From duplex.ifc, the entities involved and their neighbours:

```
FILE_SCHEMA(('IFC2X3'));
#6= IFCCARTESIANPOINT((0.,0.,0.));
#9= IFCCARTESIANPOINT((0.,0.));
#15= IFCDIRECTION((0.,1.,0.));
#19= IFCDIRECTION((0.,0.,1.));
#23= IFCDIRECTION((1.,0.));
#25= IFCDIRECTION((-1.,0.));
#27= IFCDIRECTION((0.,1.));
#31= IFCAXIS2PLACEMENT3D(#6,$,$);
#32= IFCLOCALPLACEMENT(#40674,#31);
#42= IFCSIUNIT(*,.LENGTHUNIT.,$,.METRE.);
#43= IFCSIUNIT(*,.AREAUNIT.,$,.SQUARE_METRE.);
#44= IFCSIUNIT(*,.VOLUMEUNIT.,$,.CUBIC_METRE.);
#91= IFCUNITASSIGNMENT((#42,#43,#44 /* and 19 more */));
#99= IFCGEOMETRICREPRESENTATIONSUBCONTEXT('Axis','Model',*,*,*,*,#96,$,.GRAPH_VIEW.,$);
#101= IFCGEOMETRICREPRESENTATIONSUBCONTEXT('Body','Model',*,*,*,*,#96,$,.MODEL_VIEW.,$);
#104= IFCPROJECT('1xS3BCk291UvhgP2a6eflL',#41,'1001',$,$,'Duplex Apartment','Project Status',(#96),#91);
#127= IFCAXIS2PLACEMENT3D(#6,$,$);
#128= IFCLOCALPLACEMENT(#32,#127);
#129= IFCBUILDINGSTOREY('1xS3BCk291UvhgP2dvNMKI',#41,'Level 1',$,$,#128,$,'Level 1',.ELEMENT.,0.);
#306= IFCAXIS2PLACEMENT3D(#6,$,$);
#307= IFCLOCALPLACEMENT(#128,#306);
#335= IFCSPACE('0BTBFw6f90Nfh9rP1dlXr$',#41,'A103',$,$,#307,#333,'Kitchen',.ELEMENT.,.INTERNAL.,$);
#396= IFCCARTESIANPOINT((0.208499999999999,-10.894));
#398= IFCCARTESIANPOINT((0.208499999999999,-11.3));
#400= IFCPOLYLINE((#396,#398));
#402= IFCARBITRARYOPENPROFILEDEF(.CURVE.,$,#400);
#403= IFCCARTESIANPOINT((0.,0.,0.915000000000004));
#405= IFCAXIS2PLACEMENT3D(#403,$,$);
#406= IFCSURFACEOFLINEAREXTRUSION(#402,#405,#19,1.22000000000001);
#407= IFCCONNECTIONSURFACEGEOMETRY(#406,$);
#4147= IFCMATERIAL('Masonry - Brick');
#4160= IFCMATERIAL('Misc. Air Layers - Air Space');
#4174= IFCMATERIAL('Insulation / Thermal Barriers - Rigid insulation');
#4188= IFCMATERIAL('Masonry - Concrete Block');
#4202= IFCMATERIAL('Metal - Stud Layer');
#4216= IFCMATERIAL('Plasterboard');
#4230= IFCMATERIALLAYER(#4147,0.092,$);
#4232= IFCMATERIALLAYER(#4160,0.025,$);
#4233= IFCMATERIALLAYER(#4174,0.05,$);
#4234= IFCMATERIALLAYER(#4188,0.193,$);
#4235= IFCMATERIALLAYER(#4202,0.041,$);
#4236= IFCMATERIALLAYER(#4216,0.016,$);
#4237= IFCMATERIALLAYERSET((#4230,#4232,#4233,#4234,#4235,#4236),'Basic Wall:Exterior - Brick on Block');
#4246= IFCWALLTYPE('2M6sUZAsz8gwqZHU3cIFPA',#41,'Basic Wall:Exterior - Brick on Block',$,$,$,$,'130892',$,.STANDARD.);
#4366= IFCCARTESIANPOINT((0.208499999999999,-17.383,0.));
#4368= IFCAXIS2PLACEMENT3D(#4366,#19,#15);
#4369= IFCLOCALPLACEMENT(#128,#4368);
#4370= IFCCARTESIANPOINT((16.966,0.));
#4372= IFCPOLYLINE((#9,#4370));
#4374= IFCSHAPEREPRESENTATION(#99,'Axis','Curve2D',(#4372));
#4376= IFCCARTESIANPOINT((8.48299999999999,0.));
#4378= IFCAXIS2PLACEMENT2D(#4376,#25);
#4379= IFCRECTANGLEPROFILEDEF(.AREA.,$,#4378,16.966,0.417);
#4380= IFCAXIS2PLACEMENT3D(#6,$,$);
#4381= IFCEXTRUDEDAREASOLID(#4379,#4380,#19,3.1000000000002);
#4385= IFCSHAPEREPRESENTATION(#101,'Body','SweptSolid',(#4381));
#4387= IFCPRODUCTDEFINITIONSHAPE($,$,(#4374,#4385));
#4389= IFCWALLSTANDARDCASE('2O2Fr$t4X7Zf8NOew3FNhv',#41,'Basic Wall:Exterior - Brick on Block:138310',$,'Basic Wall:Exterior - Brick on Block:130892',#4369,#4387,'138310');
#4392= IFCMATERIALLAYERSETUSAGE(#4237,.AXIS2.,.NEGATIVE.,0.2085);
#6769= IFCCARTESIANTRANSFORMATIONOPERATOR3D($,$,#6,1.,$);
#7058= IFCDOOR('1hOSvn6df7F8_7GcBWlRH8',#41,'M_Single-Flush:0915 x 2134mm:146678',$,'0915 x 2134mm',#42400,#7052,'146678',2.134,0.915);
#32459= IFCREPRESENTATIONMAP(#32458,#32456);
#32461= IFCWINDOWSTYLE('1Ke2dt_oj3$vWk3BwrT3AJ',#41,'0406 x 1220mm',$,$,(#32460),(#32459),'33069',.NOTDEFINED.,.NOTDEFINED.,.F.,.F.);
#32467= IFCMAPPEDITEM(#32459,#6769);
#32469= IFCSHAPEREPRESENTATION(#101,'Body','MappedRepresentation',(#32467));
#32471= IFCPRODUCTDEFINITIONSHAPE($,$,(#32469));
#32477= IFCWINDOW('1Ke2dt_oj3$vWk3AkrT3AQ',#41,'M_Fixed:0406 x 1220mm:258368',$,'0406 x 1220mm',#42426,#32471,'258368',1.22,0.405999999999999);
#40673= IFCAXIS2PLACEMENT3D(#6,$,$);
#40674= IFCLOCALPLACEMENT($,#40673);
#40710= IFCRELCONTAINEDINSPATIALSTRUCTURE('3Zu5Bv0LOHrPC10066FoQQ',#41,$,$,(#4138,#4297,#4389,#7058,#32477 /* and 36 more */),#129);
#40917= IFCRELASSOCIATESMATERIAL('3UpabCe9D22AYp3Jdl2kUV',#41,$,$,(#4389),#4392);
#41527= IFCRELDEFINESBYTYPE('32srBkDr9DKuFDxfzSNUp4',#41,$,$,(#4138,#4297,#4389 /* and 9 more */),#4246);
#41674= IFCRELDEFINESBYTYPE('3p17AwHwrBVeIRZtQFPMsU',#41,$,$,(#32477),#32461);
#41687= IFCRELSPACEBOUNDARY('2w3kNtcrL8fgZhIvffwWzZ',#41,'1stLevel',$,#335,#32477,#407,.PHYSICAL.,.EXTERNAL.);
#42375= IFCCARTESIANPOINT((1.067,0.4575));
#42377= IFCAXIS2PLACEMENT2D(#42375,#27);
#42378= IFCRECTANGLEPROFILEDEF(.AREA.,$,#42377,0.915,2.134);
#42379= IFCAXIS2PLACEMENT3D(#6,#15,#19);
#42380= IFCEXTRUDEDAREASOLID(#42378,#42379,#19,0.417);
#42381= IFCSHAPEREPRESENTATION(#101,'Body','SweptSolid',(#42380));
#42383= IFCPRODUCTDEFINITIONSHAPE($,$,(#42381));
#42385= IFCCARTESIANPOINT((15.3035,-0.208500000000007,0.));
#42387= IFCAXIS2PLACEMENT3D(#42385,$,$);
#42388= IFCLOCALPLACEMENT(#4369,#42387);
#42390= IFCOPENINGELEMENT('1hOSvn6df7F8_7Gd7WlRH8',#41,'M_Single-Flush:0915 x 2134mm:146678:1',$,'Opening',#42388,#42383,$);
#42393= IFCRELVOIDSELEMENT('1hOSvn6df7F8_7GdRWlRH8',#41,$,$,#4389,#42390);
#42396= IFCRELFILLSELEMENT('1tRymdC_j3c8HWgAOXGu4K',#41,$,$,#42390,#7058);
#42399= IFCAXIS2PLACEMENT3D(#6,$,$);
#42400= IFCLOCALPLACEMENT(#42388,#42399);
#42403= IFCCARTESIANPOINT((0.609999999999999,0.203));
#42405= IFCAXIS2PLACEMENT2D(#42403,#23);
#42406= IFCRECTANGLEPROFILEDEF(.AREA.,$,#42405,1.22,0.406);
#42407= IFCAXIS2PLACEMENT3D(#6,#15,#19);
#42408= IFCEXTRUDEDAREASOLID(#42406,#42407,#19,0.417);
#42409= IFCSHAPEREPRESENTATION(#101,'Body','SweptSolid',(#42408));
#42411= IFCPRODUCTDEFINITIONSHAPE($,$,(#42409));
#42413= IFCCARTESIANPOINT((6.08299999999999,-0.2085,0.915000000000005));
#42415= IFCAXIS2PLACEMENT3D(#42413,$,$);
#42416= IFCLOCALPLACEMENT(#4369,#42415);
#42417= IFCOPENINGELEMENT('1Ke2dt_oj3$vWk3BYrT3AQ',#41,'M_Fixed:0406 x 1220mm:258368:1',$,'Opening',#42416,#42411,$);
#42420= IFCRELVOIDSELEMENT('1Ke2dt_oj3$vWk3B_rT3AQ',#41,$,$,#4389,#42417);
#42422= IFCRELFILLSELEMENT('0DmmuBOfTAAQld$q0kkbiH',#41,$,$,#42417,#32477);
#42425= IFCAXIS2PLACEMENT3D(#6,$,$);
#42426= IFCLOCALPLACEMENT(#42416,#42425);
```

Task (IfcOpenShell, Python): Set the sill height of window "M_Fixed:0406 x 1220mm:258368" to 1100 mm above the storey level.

```python
import numpy as np
import ifcopenshell
import ifcopenshell.api.geometry
import ifcopenshell.geom
import ifcopenshell.util.element
import ifcopenshell.util.placement
import ifcopenshell.util.shape
import ifcopenshell.util.unit

model = ifcopenshell.open("duplex.ifc")
unit_scale = ifcopenshell.util.unit.calculate_unit_scale(model)

window = model.by_guid("1Ke2dt_oj3$vWk3AkrT3AQ")
opening = window.FillsVoids[0].RelatingOpeningElement
storey = ifcopenshell.util.element.get_container(window, ifc_class="IfcBuildingStorey")
level = ifcopenshell.util.placement.get_local_placement(storey.ObjectPlacement)[2, 3]

# The opening's origin need not be at the sill, so measure its lowest point.
shape = ifcopenshell.geom.create_shape(ifcopenshell.geom.settings(), opening)
bottom = ifcopenshell.util.shape.get_shape_bottom_elevation(shape, shape.geometry) / unit_scale
dz = level + 1.1 / unit_scale - bottom

shift = np.array([0.0, 0.0, dz])
# The window is placed relative to its opening, so it follows when the opening moves.
matrix = ifcopenshell.util.placement.get_local_placement(opening.ObjectPlacement)
matrix[:3, 3] += shift
ifcopenshell.api.geometry.edit_object_placement(
    model, product=opening, matrix=matrix, is_si=False, should_transform_children=True
)

# Space boundary surfaces are stored in each space's coordinates; move them too.
for rel in window.ProvidesBoundaries:
    if not rel.ConnectionGeometry:
        continue
    surface = rel.ConnectionGeometry.SurfaceOnRelatingElement
    space_matrix = ifcopenshell.util.placement.get_local_placement(rel.RelatingSpace.ObjectPlacement)
    point = np.array(surface.Position.Location.Coordinates) + space_matrix[:3, :3].T @ shift
    surface.Position = model.createIfcAxis2Placement3D(
        model.createIfcCartesianPoint(point.tolist()), surface.Position.Axis, surface.Position.RefDirection
    )

print(f"moved by {dz * unit_scale:+.3f} m")

model.write("duplex_edited.ifc")
```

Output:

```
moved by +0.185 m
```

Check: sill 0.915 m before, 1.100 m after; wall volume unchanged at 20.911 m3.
